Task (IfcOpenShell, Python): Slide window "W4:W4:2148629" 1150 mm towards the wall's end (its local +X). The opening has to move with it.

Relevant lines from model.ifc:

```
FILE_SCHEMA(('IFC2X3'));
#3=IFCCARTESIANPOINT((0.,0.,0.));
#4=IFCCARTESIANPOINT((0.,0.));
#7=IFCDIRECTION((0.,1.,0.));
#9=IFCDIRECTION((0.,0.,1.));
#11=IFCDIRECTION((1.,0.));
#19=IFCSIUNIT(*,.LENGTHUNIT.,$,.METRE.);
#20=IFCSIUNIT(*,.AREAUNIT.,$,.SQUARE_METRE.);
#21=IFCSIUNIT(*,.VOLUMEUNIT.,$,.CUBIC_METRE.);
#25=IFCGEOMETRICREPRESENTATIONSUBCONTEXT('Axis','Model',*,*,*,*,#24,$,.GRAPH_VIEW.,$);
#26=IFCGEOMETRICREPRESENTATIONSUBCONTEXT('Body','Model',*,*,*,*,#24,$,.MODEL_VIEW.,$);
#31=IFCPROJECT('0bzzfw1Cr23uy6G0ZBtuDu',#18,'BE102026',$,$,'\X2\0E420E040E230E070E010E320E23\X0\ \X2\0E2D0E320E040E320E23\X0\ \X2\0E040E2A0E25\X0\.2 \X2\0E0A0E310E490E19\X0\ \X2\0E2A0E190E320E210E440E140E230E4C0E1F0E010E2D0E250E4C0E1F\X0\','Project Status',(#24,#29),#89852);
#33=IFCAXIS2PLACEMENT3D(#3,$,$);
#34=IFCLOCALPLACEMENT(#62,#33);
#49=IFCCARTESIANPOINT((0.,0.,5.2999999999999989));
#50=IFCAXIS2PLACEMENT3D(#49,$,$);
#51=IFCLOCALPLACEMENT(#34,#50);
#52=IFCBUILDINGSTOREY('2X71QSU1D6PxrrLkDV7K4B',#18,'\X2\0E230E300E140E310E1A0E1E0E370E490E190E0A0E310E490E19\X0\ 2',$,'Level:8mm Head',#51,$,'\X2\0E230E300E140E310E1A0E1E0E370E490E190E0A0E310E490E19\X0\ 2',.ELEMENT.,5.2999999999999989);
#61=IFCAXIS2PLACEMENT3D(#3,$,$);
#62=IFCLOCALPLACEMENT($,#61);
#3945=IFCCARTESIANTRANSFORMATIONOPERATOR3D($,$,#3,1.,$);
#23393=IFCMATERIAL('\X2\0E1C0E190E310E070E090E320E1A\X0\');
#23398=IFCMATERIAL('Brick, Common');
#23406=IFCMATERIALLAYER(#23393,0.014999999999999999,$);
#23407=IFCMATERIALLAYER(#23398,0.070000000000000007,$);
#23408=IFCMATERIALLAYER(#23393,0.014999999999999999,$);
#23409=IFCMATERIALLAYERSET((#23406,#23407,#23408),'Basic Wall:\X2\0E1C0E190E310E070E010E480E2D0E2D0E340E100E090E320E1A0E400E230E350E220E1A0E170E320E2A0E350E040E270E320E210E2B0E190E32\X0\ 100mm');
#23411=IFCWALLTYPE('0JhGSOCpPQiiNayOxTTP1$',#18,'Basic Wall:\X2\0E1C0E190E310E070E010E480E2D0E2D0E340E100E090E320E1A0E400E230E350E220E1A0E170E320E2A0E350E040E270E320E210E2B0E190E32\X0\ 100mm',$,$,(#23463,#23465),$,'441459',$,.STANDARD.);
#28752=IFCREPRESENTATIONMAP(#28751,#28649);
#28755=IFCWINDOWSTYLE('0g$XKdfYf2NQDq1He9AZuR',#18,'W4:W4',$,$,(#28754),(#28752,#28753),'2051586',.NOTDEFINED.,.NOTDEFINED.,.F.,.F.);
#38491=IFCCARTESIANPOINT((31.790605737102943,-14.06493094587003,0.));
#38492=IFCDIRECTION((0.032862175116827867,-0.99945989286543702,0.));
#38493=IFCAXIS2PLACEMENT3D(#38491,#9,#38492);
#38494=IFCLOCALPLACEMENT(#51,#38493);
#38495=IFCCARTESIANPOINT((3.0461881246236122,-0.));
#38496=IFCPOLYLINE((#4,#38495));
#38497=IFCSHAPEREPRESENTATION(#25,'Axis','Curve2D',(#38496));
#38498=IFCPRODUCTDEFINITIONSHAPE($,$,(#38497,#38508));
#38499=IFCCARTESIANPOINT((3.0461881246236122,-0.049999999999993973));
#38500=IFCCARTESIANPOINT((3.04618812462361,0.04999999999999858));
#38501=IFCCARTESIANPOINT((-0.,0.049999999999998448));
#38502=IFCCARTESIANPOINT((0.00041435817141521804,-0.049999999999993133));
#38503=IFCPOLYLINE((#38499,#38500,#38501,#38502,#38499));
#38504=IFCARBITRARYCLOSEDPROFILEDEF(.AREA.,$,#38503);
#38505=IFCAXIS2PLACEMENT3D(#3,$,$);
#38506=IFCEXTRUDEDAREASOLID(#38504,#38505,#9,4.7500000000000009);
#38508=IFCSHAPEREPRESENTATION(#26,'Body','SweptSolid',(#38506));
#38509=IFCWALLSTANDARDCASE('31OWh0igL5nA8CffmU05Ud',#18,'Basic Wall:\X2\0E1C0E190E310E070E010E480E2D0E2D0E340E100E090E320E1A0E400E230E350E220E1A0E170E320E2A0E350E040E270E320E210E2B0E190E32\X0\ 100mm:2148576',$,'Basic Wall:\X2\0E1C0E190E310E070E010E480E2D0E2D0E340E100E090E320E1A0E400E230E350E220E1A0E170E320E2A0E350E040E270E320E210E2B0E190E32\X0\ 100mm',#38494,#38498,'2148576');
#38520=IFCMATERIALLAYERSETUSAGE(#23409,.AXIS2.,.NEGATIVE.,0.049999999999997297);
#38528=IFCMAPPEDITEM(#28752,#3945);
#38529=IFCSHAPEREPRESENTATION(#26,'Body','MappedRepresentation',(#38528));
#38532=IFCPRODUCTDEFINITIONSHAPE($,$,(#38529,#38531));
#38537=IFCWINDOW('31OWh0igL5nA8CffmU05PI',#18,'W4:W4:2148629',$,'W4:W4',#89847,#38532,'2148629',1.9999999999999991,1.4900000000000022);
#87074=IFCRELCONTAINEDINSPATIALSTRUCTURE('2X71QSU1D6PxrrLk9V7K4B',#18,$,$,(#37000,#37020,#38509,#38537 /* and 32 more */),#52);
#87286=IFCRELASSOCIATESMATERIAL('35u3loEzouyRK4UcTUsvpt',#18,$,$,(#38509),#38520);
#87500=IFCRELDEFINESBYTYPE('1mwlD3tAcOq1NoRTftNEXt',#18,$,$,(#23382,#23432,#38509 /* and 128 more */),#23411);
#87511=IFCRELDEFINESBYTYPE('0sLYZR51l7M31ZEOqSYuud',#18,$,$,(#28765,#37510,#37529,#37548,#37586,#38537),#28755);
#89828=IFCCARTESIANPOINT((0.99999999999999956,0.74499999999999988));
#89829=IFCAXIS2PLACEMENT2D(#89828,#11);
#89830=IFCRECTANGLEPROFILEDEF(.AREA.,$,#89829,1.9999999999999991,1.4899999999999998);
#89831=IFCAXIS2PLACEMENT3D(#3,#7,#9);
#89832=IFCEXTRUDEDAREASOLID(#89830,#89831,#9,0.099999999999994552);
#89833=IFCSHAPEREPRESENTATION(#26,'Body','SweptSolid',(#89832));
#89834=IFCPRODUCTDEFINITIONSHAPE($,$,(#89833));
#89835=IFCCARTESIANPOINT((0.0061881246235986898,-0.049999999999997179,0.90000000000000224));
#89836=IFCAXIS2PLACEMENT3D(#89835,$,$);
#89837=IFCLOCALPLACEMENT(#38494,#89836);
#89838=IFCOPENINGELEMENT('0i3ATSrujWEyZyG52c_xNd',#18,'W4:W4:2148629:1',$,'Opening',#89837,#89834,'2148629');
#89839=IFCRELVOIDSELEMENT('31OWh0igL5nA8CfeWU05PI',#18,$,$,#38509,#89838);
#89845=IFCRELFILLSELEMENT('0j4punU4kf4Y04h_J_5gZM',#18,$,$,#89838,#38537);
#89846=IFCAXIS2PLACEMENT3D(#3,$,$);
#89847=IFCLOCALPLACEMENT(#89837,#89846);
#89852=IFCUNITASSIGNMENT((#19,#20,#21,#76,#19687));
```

```python
import ifcopenshell
import ifcopenshell.api.geometry
import ifcopenshell.util.placement

model = ifcopenshell.open("model.ifc")

window = model.by_id(38537)
opening = window.FillsVoids[0].RelatingOpeningElement
wall = opening.VoidsElements[0].RelatingBuildingElement

wall_matrix = ifcopenshell.util.placement.get_local_placement(wall.ObjectPlacement)
shift = wall_matrix[:3, 0] * 1.15
before = ifcopenshell.util.placement.get_local_placement(window.ObjectPlacement)[:3, 3].copy()

# The window is placed relative to its opening, so it follows when the opening moves.
matrix = ifcopenshell.util.placement.get_local_placement(opening.ObjectPlacement)
matrix[:3, 3] += shift
ifcopenshell.api.geometry.edit_object_placement(
    model, product=opening, matrix=matrix, is_si=False, should_transform_children=True
)

after = ifcopenshell.util.placement.get_local_placement(window.ObjectPlacement)[:3, 3]
print("window moved by", (after - before).round(3) + 0.0)

model.write("model-out.ifc")
```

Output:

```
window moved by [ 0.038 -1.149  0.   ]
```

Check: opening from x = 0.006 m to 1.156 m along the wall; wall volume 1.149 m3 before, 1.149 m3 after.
